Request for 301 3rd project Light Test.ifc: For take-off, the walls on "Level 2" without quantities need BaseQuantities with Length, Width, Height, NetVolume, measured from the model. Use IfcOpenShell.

First a look at what the model holds.

```python
import ifcopenshell
import ifcopenshell.util.element
import ifcopenshell.util.unit

model = ifcopenshell.open("301 3rd project Light Test.ifc")
print(model.schema)
for unit_type in ("LENGTHUNIT", "AREAUNIT", "VOLUMEUNIT"):
    print(unit_type, ifcopenshell.util.unit.calculate_unit_scale(model, unit_type))
storey = next(s for s in model.by_type("IfcBuildingStorey") if s.Name == "Level 2")
walls = [e for e in ifcopenshell.util.element.get_decomposition(storey) if e.is_a("IfcWall")]
for e in sorted(walls, key=lambda e: e.id()):
    print(e.id(), e.is_a(), e.Name, list(ifcopenshell.util.element.get_psets(e, qtos_only=True)), sep=" | ")
```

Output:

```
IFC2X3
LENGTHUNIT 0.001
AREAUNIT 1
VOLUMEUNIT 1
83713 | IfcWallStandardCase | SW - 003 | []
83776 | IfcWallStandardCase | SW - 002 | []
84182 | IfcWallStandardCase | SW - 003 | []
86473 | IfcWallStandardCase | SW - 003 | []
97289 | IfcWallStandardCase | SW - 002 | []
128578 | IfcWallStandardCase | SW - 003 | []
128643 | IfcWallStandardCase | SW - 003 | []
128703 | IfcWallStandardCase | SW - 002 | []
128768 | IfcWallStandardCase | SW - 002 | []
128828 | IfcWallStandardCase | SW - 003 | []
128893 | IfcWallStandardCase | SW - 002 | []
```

```python
import ifcopenshell
import ifcopenshell.api.pset
import ifcopenshell.geom
import ifcopenshell.util.element
import ifcopenshell.util.shape
import ifcopenshell.util.unit

model = ifcopenshell.open("301 3rd project Light Test.ifc")
unit_scale = ifcopenshell.util.unit.calculate_unit_scale(model)
volume_scale = ifcopenshell.util.unit.calculate_unit_scale(model, "VOLUMEUNIT")
settings = ifcopenshell.geom.settings()

storey = next(s for s in model.by_type("IfcBuildingStorey") if s.Name == "Level 2")
walls = [e for e in ifcopenshell.util.element.get_decomposition(storey) if e.is_a("IfcWall")]

for e in sorted(walls, key=lambda e: e.id()):
    if ifcopenshell.util.element.get_psets(e, qtos_only=True, should_inherit=False):
        continue
    # Geometry comes back in metres, in the element's own axes.
    shape = ifcopenshell.geom.create_shape(settings, e)
    values = {
        "Length": ifcopenshell.util.shape.get_x(shape.geometry) / unit_scale,
        "Width": ifcopenshell.util.shape.get_y(shape.geometry) / unit_scale,
        "Height": ifcopenshell.util.shape.get_z(shape.geometry) / unit_scale,
        "NetVolume": ifcopenshell.util.shape.get_volume(shape.geometry) / volume_scale,
    }
    qto = ifcopenshell.api.pset.add_qto(model, product=e, name="BaseQuantities")
    ifcopenshell.api.pset.edit_qto(model, qto=qto, properties=values)
    print(e.id(), {k: round(v, 3) for k, v in values.items()})

model.write("301 3rd project Light Test_updated.ifc")
```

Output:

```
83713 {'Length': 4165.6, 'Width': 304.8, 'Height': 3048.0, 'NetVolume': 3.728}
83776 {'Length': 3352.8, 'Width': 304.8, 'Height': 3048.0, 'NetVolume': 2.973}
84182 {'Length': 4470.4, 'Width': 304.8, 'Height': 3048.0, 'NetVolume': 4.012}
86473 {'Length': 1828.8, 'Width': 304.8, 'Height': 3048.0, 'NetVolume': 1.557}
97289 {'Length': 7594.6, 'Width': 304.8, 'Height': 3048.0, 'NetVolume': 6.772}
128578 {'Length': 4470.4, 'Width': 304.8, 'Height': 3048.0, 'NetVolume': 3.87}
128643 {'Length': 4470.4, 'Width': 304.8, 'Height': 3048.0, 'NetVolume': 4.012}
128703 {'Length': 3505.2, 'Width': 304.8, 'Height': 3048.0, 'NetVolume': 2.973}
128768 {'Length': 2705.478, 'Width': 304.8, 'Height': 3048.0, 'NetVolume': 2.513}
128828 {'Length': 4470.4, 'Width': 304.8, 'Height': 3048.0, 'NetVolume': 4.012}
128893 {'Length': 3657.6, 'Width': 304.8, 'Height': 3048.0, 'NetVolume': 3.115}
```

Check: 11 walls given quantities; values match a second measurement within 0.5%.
